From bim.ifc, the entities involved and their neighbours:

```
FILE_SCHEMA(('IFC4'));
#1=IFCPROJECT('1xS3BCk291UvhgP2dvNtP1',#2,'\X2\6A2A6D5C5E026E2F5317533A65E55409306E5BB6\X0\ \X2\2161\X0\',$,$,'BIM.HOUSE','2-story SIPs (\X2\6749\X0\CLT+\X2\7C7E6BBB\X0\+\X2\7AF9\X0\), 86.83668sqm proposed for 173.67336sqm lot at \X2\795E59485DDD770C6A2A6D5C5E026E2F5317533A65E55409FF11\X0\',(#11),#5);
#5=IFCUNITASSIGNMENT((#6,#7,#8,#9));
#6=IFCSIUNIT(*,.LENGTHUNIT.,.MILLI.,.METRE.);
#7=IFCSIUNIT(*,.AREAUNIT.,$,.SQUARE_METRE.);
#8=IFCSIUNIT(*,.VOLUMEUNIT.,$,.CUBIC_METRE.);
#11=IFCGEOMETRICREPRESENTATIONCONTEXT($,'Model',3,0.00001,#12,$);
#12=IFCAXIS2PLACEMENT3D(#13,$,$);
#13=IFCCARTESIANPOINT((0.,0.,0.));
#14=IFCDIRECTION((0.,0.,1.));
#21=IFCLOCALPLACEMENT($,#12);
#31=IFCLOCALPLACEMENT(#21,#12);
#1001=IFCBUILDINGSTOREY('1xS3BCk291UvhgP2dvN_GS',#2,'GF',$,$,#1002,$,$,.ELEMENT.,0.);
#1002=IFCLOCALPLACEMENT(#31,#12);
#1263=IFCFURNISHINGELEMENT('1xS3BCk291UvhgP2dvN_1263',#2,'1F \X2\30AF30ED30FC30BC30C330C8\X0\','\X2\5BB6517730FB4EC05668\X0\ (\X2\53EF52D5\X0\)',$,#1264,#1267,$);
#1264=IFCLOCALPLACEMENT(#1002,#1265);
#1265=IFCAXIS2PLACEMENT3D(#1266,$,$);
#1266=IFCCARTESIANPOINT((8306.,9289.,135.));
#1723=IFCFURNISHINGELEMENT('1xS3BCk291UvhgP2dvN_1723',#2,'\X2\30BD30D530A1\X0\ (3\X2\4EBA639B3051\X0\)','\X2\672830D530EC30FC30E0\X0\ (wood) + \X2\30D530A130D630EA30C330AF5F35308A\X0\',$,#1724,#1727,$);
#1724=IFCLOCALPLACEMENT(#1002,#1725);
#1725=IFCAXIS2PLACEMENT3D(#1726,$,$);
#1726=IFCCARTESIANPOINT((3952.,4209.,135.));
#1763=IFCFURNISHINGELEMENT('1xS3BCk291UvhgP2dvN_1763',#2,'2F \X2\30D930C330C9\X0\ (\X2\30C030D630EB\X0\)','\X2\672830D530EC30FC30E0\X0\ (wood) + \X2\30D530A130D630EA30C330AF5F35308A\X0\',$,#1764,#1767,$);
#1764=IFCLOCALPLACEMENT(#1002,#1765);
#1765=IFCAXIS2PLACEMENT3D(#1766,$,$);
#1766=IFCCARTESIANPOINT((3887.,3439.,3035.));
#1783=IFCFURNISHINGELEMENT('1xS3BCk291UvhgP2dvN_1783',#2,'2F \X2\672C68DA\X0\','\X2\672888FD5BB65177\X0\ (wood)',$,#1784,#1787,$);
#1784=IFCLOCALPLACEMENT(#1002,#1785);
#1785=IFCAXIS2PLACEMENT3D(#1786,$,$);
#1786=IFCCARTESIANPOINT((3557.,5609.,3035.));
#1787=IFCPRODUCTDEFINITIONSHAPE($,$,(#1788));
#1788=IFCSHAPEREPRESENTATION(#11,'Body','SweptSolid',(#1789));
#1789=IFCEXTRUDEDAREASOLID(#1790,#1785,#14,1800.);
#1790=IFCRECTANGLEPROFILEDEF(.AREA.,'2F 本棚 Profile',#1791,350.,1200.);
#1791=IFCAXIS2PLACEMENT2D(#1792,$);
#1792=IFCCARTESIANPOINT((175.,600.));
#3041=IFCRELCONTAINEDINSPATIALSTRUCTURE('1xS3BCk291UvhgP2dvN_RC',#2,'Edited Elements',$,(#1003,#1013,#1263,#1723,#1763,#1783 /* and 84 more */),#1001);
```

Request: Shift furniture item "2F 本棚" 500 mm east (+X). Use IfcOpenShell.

```python
import ifcopenshell
import ifcopenshell.api.geometry
import ifcopenshell.util.placement

model = ifcopenshell.open("bim.ifc")

item = model.by_guid("1xS3BCk291UvhgP2dvN_1783")
matrix = ifcopenshell.util.placement.get_local_placement(item.ObjectPlacement)
matrix[0, 3] += 500.0
ifcopenshell.api.geometry.edit_object_placement(model, product=item, matrix=matrix, is_si=False)

print(ifcopenshell.util.placement.get_local_placement(item.ObjectPlacement).round(3) + 0.0)

model.write("bim_edited.ifc")
```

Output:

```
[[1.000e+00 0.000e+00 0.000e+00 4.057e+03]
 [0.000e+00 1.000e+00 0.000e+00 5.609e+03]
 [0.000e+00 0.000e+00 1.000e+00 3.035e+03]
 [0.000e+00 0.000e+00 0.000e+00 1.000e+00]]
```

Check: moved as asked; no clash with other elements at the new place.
